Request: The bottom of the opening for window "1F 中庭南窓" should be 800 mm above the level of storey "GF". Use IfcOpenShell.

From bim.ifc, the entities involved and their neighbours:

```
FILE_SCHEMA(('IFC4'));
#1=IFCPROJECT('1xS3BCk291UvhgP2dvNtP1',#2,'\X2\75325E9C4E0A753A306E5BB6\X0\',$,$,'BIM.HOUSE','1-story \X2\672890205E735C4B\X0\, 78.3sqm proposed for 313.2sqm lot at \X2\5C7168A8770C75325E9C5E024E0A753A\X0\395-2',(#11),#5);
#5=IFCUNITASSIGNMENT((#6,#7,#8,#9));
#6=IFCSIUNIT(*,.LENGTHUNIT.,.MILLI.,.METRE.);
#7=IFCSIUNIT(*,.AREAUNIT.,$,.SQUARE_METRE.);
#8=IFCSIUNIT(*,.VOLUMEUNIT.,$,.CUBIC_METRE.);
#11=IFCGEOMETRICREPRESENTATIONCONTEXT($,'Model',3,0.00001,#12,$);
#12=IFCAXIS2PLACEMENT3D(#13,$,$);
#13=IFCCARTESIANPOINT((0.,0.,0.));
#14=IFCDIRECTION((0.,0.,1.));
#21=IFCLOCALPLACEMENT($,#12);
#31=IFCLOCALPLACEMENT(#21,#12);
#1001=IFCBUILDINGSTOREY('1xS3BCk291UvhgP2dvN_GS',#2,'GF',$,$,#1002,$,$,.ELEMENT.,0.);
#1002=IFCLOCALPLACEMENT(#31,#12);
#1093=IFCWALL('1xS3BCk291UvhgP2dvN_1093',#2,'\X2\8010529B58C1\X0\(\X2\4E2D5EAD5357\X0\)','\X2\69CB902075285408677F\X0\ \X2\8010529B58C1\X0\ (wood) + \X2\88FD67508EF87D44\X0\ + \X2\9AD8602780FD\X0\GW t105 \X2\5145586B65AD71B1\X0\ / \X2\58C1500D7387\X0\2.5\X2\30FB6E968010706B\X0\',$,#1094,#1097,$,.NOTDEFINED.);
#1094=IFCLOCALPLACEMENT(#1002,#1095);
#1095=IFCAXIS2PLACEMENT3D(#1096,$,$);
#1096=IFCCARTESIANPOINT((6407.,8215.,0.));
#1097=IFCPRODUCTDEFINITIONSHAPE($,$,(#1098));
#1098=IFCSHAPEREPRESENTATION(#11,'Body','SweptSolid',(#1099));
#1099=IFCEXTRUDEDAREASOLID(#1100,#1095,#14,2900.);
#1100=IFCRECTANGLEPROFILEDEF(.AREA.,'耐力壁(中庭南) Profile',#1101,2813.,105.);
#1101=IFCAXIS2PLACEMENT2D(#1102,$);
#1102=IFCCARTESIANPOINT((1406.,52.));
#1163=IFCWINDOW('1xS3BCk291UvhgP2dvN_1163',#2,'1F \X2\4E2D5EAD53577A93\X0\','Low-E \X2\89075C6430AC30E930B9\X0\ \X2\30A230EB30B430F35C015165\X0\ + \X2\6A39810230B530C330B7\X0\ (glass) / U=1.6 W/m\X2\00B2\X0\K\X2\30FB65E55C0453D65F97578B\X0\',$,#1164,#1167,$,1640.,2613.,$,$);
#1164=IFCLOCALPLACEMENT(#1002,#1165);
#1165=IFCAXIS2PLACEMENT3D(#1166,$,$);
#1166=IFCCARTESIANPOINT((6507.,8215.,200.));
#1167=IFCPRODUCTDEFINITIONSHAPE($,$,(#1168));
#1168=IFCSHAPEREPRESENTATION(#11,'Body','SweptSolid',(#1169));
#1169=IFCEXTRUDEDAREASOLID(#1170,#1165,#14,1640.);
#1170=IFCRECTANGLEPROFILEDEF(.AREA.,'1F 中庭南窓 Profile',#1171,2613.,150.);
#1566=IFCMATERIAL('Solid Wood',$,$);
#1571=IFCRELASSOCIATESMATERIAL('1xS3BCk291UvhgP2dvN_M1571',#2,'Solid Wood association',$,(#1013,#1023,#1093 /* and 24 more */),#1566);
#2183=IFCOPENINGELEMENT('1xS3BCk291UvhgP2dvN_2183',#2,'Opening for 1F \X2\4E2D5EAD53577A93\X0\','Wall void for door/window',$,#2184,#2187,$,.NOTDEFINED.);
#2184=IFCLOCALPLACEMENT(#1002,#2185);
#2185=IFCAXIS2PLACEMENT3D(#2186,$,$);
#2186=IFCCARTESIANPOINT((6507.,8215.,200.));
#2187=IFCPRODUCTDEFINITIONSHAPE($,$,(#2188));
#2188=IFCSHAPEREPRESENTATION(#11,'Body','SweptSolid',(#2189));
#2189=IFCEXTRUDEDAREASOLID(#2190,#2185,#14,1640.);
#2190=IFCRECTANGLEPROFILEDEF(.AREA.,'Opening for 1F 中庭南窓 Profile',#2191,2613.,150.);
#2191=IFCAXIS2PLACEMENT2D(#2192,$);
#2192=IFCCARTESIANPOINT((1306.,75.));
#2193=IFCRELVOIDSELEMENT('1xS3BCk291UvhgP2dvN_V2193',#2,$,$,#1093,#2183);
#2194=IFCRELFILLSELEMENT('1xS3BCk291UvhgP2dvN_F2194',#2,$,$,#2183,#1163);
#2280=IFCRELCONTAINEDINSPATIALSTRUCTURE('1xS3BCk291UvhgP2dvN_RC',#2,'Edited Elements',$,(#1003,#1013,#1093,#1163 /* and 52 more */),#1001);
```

```python
import numpy as np
import ifcopenshell
import ifcopenshell.api.geometry
import ifcopenshell.geom
import ifcopenshell.util.element
import ifcopenshell.util.placement
import ifcopenshell.util.shape
import ifcopenshell.util.unit

model = ifcopenshell.open("bim.ifc")
unit_scale = ifcopenshell.util.unit.calculate_unit_scale(model)

window = model.by_guid("1xS3BCk291UvhgP2dvN_1163")
opening = window.FillsVoids[0].RelatingOpeningElement
storey = ifcopenshell.util.element.get_container(window, ifc_class="IfcBuildingStorey")
level = ifcopenshell.util.placement.get_local_placement(storey.ObjectPlacement)[2, 3]

# The opening's origin need not be at the sill, so measure its lowest point.
shape = ifcopenshell.geom.create_shape(ifcopenshell.geom.settings(), opening)
bottom = ifcopenshell.util.shape.get_shape_bottom_elevation(shape, shape.geometry) / unit_scale
dz = level + 0.8 / unit_scale - bottom

shift = np.array([0.0, 0.0, dz])
# The window is not placed relative to its opening, so move both.
for product in (opening, window):
    matrix = ifcopenshell.util.placement.get_local_placement(product.ObjectPlacement)
    matrix[:3, 3] += shift
    ifcopenshell.api.geometry.edit_object_placement(model, product=product, matrix=matrix, is_si=False)

print(f"moved by {dz * unit_scale:+.3f} m")

model.write("bim_rev.ifc")
```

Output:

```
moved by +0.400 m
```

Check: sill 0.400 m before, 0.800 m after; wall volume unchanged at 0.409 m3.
